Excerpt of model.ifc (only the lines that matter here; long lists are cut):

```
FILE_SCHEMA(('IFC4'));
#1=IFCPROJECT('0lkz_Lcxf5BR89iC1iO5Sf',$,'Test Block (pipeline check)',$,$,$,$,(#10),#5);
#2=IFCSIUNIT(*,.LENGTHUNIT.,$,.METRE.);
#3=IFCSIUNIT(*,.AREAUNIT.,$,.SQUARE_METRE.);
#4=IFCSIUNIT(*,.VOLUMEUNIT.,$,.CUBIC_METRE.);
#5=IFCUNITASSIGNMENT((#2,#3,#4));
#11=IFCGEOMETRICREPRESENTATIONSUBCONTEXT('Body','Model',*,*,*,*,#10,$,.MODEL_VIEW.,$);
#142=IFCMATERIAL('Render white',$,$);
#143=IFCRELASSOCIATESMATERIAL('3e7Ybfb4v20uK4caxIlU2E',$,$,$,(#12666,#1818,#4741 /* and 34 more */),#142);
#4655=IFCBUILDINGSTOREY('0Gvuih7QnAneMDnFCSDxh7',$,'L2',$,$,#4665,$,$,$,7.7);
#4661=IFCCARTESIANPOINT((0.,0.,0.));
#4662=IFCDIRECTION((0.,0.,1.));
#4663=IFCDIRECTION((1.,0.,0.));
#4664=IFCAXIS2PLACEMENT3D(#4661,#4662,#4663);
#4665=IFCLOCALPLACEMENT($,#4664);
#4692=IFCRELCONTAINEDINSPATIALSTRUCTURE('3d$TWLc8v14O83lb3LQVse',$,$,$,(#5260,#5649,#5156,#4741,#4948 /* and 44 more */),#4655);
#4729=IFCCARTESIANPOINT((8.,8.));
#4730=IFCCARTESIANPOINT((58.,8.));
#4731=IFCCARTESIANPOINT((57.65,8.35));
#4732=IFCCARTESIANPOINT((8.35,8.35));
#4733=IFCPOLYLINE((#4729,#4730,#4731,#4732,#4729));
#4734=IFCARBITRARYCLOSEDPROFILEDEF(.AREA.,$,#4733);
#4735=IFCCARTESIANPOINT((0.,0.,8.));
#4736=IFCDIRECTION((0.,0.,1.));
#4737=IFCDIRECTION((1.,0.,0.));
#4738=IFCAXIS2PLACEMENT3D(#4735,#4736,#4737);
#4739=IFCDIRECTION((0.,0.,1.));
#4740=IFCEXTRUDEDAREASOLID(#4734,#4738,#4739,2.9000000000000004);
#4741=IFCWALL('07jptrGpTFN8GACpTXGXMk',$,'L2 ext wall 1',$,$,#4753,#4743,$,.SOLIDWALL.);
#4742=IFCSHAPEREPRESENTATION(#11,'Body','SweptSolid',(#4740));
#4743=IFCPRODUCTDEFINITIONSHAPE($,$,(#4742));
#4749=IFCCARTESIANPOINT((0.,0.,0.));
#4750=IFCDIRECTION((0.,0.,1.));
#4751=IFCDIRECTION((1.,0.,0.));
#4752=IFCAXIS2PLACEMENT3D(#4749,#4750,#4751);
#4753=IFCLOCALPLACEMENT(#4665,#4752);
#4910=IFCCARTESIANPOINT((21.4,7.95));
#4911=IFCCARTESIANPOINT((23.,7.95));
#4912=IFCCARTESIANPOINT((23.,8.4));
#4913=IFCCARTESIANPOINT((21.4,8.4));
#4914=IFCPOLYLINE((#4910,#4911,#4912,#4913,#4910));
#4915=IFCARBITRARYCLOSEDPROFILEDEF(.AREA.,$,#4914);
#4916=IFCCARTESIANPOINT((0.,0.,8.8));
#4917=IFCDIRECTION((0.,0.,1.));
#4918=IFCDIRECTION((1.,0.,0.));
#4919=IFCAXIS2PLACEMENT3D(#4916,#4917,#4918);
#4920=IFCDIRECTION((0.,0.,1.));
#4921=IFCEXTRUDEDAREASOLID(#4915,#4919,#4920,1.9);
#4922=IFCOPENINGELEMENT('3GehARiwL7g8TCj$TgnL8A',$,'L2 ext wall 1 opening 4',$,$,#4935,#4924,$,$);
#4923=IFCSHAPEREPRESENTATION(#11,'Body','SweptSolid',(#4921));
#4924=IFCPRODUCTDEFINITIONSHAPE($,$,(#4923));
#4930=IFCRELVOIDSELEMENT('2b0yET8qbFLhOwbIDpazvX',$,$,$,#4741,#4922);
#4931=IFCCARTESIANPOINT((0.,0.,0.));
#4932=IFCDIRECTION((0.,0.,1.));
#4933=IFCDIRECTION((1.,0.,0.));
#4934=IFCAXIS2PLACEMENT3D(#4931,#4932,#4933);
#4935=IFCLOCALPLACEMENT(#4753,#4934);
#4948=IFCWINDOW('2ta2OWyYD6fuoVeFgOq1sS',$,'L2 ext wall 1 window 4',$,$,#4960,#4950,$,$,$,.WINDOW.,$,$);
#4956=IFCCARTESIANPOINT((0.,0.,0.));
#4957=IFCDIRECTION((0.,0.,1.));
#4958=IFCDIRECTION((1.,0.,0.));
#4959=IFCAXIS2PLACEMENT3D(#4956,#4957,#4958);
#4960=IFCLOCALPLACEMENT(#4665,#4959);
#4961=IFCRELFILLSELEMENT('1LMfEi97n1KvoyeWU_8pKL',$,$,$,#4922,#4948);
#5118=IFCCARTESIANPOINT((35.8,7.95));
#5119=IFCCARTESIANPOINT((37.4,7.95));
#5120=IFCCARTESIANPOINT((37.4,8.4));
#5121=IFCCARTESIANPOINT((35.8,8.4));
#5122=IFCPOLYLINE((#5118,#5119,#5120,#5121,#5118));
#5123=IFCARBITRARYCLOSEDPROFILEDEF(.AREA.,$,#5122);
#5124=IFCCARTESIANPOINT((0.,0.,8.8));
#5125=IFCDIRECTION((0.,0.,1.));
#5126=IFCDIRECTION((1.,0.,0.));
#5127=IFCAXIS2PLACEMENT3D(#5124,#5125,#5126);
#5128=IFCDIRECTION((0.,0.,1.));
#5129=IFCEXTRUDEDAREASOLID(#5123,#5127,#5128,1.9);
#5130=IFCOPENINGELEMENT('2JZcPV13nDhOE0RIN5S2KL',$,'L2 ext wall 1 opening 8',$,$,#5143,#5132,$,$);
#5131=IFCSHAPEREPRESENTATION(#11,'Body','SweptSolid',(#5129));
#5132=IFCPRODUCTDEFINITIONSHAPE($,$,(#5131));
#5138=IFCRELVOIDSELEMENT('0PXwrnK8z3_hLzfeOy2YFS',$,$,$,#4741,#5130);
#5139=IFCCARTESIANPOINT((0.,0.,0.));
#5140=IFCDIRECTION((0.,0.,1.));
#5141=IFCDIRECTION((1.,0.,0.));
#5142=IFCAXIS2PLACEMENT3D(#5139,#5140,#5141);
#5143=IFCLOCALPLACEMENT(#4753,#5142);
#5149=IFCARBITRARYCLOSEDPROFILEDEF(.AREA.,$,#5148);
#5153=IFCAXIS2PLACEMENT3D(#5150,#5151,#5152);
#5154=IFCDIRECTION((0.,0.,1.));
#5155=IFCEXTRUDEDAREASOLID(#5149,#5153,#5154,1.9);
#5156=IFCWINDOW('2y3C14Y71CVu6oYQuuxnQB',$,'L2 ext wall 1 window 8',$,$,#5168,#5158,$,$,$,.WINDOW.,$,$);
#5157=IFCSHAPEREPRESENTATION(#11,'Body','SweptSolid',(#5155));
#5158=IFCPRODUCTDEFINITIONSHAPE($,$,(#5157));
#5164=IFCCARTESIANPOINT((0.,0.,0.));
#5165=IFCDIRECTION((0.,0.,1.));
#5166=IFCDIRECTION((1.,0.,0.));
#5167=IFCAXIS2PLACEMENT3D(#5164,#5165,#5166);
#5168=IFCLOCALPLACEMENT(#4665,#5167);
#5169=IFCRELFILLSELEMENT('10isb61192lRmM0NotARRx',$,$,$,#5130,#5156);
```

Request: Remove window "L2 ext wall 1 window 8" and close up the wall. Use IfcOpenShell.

```python
import ifcopenshell
import ifcopenshell.api.feature
import ifcopenshell.api.root
import ifcopenshell.geom
import ifcopenshell.util.shape

model = ifcopenshell.open("model.ifc")
settings = ifcopenshell.geom.settings()


def volume(element):
    """Net volume in cubic metres, openings subtracted."""
    shape = ifcopenshell.geom.create_shape(settings, element)
    return ifcopenshell.util.shape.get_volume(shape.geometry)


window = model.by_id(5156)
opening = window.FillsVoids[0].RelatingOpeningElement
wall = opening.VoidsElements[0].RelatingBuildingElement
before = volume(wall)

ifcopenshell.api.root.remove_product(model, product=window)
ifcopenshell.api.feature.remove_feature(model, feature=opening)

after = volume(wall)

print(f"wall volume {before:.3f} -> {after:.3f} m3")

model.write("model_rev.ifc")
```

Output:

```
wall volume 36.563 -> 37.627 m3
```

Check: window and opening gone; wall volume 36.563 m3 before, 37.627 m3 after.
